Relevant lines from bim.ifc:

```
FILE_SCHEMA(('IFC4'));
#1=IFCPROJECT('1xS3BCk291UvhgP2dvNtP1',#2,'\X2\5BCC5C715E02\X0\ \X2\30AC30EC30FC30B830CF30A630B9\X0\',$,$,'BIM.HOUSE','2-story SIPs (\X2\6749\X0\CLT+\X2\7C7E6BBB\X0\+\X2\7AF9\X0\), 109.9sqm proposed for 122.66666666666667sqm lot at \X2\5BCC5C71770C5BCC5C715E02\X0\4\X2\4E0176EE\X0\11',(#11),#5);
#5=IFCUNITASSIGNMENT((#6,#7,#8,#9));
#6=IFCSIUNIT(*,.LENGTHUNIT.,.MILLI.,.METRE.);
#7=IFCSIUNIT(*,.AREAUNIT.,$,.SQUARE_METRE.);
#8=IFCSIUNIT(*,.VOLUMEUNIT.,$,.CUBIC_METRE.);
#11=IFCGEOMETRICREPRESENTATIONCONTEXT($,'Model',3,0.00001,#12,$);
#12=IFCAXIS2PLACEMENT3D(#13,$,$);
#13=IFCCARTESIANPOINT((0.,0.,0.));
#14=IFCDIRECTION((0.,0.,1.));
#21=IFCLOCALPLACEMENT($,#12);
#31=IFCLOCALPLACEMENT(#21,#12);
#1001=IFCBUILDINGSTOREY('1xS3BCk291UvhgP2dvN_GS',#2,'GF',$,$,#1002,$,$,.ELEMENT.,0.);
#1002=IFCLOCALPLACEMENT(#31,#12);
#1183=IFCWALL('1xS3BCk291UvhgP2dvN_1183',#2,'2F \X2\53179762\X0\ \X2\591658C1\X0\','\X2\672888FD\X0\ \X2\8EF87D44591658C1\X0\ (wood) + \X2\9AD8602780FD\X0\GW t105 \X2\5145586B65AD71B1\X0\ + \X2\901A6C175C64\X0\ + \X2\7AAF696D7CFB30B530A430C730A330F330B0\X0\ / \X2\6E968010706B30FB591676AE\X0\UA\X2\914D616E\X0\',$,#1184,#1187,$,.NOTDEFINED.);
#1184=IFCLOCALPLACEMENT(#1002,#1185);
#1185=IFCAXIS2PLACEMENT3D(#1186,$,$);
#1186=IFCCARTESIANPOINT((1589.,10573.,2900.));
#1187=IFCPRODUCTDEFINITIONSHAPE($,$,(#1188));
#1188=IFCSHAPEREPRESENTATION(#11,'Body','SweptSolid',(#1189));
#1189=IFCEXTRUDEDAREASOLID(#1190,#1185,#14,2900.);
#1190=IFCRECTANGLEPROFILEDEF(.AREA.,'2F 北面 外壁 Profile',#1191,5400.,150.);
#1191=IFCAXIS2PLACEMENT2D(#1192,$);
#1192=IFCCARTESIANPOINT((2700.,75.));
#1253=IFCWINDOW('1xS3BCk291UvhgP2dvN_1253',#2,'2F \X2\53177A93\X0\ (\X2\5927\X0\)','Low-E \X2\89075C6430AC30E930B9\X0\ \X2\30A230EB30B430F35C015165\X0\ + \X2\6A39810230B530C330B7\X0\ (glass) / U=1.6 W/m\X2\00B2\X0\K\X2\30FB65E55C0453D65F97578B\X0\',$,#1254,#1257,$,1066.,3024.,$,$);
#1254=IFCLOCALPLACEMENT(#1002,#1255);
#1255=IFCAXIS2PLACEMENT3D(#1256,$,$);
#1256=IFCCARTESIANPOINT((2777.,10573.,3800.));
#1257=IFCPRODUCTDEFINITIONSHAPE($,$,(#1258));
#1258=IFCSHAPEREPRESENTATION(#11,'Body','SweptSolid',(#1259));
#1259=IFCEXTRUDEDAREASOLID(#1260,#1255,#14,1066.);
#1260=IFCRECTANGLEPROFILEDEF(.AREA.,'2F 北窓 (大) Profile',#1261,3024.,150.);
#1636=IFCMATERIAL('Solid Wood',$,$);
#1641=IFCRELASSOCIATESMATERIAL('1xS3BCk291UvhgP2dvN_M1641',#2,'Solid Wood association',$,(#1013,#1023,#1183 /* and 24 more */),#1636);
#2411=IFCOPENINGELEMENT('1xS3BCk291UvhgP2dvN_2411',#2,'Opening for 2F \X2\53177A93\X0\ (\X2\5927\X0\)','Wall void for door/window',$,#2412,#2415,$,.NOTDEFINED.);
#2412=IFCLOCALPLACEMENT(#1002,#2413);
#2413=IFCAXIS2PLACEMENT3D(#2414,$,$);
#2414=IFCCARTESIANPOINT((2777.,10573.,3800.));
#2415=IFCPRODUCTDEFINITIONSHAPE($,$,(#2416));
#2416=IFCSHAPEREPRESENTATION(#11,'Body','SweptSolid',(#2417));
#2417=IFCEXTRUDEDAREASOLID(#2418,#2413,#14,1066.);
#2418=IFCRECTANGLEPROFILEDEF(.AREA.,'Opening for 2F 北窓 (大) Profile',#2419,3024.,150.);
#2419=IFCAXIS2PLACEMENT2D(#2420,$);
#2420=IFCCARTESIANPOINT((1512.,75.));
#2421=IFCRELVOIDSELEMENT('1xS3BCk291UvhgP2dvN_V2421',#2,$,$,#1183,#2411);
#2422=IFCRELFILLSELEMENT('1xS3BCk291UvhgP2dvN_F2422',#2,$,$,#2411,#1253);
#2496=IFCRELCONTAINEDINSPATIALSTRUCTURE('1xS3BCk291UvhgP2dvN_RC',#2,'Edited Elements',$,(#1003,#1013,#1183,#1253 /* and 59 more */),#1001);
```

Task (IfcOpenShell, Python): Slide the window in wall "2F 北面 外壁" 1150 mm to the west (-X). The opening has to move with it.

```python
import ifcopenshell
import ifcopenshell.api.geometry
import ifcopenshell.util.placement

model = ifcopenshell.open("bim.ifc")

window = model.by_guid("1xS3BCk291UvhgP2dvN_1253")
opening = window.FillsVoids[0].RelatingOpeningElement
wall = opening.VoidsElements[0].RelatingBuildingElement

wall_matrix = ifcopenshell.util.placement.get_local_placement(wall.ObjectPlacement)
shift = wall_matrix[:3, 0] * -1150.0
before = ifcopenshell.util.placement.get_local_placement(window.ObjectPlacement)[:3, 3].copy()

# The window is not placed relative to its opening, so move both.
for product in (opening, window):
    matrix = ifcopenshell.util.placement.get_local_placement(product.ObjectPlacement)
    matrix[:3, 3] += shift
    ifcopenshell.api.geometry.edit_object_placement(model, product=product, matrix=matrix, is_si=False)

after = ifcopenshell.util.placement.get_local_placement(window.ObjectPlacement)[:3, 3]
print("window moved by", (after - before).round(3) + 0.0)

model.write("bim_rev.ifc")
```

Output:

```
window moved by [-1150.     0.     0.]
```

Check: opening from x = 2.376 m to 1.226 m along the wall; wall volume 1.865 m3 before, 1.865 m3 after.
